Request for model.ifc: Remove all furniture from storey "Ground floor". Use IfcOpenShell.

First a look at what the model holds.

```python
import ifcopenshell
import ifcopenshell.util.element

model = ifcopenshell.open("model.ifc")
print(model.schema)
storey = next(s for s in model.by_type("IfcBuildingStorey") if s.Name == "Ground floor")
furniture = [e for e in ifcopenshell.util.element.get_decomposition(storey) if e.is_a("IfcFurnishingElement")]
seen = {}
for e in furniture:
    element_type = ifcopenshell.util.element.get_type(e)
    name = element_type.Name if element_type not in (None, e) else None
    seen[name] = seen.get(name, 0) + 1
for name, count in sorted(seen.items(), key=str):
    print(count, "x", name)
```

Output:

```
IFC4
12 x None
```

```python
import ifcopenshell
import ifcopenshell.api.root
import ifcopenshell.util.element

model = ifcopenshell.open("model.ifc")

storey = next(s for s in model.by_type("IfcBuildingStorey") if s.Name == "Ground floor")
furniture = [e for e in ifcopenshell.util.element.get_decomposition(storey) if e.is_a("IfcFurnishingElement")]

for e in furniture:
    ifcopenshell.api.root.remove_product(model, product=e)
print(len(furniture), "removed")

model.write("model_v2.ifc")
```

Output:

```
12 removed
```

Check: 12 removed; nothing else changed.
